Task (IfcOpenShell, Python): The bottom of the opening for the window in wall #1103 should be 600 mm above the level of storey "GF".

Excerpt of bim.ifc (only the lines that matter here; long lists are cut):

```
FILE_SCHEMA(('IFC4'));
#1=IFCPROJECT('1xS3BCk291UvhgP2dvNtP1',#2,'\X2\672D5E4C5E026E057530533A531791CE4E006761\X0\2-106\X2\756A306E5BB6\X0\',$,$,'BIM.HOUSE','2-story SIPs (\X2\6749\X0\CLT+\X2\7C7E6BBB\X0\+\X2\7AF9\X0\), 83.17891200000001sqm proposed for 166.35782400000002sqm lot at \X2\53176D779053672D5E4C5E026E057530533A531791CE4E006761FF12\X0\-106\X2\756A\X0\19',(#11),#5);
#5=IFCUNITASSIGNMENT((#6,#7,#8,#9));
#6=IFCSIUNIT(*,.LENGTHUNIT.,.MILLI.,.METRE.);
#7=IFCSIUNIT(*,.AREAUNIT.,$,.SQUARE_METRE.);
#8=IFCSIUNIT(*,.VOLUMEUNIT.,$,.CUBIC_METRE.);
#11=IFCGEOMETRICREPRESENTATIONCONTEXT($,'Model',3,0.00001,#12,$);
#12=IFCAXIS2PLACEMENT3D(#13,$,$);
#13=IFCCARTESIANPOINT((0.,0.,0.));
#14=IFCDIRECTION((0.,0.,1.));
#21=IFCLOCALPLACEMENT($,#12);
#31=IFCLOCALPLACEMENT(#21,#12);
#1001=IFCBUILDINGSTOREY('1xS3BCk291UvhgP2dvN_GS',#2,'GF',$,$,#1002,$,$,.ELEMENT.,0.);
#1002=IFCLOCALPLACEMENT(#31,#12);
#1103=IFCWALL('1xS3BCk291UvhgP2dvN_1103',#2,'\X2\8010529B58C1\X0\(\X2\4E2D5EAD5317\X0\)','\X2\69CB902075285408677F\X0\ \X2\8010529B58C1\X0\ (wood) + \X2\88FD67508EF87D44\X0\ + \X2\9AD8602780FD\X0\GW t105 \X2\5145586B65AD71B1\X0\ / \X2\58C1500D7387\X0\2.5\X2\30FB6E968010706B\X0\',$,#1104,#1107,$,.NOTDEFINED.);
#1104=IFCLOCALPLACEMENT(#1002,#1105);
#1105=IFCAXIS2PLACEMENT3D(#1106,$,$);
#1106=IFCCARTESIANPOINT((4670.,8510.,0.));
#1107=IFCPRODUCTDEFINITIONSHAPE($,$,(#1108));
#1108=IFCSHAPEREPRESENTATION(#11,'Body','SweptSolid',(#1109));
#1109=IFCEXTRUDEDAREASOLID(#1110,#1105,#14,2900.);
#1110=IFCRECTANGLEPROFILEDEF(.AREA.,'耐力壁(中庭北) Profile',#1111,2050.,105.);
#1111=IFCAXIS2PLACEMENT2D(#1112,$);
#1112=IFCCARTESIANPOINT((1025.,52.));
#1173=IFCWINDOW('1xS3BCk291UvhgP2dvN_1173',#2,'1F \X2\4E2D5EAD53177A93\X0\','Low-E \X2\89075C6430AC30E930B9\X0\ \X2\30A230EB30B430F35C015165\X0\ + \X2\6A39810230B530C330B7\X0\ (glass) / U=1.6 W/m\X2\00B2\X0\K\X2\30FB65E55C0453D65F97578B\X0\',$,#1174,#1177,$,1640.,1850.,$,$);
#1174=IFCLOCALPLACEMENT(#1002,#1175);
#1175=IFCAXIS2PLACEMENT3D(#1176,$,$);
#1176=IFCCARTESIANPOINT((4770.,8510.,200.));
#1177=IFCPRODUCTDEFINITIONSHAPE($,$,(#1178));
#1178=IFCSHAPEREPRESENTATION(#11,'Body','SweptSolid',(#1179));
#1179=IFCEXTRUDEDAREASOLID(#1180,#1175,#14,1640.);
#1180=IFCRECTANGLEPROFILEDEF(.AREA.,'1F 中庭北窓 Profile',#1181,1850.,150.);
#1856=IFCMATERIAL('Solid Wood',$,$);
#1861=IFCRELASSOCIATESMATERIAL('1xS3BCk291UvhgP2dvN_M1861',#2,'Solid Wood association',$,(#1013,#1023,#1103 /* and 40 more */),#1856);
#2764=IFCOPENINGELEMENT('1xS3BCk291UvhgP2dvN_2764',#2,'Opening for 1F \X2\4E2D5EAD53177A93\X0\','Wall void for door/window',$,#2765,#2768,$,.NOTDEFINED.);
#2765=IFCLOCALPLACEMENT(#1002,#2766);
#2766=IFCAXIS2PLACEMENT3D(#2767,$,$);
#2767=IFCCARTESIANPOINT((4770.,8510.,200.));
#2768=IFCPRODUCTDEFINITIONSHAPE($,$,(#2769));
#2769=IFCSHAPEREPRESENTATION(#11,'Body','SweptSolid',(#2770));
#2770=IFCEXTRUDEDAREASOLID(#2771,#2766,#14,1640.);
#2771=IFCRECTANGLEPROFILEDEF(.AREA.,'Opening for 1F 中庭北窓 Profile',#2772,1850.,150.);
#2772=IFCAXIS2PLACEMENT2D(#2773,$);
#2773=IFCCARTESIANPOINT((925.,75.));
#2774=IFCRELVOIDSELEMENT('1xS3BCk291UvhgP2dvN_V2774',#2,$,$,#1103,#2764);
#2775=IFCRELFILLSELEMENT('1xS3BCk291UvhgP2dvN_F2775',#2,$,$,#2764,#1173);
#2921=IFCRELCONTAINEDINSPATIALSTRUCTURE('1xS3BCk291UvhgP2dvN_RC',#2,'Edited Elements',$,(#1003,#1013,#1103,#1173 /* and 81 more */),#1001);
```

```python
import numpy as np
import ifcopenshell
import ifcopenshell.api.geometry
import ifcopenshell.geom
import ifcopenshell.util.element
import ifcopenshell.util.placement
import ifcopenshell.util.shape
import ifcopenshell.util.unit

model = ifcopenshell.open("bim.ifc")
unit_scale = ifcopenshell.util.unit.calculate_unit_scale(model)

window = model.by_guid("1xS3BCk291UvhgP2dvN_1173")
opening = window.FillsVoids[0].RelatingOpeningElement
storey = ifcopenshell.util.element.get_container(window, ifc_class="IfcBuildingStorey")
level = ifcopenshell.util.placement.get_local_placement(storey.ObjectPlacement)[2, 3]

# The opening's origin need not be at the sill, so measure its lowest point.
shape = ifcopenshell.geom.create_shape(ifcopenshell.geom.settings(), opening)
bottom = ifcopenshell.util.shape.get_shape_bottom_elevation(shape, shape.geometry) / unit_scale
dz = level + 0.6 / unit_scale - bottom

shift = np.array([0.0, 0.0, dz])
# The window is not placed relative to its opening, so move both.
for product in (opening, window):
    matrix = ifcopenshell.util.placement.get_local_placement(product.ObjectPlacement)
    matrix[:3, 3] += shift
    ifcopenshell.api.geometry.edit_object_placement(model, product=product, matrix=matrix, is_si=False)

print(f"moved by {dz * unit_scale:+.3f} m")

model.write("bim_v2.ifc")
```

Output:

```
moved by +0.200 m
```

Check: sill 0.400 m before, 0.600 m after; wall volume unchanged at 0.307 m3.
